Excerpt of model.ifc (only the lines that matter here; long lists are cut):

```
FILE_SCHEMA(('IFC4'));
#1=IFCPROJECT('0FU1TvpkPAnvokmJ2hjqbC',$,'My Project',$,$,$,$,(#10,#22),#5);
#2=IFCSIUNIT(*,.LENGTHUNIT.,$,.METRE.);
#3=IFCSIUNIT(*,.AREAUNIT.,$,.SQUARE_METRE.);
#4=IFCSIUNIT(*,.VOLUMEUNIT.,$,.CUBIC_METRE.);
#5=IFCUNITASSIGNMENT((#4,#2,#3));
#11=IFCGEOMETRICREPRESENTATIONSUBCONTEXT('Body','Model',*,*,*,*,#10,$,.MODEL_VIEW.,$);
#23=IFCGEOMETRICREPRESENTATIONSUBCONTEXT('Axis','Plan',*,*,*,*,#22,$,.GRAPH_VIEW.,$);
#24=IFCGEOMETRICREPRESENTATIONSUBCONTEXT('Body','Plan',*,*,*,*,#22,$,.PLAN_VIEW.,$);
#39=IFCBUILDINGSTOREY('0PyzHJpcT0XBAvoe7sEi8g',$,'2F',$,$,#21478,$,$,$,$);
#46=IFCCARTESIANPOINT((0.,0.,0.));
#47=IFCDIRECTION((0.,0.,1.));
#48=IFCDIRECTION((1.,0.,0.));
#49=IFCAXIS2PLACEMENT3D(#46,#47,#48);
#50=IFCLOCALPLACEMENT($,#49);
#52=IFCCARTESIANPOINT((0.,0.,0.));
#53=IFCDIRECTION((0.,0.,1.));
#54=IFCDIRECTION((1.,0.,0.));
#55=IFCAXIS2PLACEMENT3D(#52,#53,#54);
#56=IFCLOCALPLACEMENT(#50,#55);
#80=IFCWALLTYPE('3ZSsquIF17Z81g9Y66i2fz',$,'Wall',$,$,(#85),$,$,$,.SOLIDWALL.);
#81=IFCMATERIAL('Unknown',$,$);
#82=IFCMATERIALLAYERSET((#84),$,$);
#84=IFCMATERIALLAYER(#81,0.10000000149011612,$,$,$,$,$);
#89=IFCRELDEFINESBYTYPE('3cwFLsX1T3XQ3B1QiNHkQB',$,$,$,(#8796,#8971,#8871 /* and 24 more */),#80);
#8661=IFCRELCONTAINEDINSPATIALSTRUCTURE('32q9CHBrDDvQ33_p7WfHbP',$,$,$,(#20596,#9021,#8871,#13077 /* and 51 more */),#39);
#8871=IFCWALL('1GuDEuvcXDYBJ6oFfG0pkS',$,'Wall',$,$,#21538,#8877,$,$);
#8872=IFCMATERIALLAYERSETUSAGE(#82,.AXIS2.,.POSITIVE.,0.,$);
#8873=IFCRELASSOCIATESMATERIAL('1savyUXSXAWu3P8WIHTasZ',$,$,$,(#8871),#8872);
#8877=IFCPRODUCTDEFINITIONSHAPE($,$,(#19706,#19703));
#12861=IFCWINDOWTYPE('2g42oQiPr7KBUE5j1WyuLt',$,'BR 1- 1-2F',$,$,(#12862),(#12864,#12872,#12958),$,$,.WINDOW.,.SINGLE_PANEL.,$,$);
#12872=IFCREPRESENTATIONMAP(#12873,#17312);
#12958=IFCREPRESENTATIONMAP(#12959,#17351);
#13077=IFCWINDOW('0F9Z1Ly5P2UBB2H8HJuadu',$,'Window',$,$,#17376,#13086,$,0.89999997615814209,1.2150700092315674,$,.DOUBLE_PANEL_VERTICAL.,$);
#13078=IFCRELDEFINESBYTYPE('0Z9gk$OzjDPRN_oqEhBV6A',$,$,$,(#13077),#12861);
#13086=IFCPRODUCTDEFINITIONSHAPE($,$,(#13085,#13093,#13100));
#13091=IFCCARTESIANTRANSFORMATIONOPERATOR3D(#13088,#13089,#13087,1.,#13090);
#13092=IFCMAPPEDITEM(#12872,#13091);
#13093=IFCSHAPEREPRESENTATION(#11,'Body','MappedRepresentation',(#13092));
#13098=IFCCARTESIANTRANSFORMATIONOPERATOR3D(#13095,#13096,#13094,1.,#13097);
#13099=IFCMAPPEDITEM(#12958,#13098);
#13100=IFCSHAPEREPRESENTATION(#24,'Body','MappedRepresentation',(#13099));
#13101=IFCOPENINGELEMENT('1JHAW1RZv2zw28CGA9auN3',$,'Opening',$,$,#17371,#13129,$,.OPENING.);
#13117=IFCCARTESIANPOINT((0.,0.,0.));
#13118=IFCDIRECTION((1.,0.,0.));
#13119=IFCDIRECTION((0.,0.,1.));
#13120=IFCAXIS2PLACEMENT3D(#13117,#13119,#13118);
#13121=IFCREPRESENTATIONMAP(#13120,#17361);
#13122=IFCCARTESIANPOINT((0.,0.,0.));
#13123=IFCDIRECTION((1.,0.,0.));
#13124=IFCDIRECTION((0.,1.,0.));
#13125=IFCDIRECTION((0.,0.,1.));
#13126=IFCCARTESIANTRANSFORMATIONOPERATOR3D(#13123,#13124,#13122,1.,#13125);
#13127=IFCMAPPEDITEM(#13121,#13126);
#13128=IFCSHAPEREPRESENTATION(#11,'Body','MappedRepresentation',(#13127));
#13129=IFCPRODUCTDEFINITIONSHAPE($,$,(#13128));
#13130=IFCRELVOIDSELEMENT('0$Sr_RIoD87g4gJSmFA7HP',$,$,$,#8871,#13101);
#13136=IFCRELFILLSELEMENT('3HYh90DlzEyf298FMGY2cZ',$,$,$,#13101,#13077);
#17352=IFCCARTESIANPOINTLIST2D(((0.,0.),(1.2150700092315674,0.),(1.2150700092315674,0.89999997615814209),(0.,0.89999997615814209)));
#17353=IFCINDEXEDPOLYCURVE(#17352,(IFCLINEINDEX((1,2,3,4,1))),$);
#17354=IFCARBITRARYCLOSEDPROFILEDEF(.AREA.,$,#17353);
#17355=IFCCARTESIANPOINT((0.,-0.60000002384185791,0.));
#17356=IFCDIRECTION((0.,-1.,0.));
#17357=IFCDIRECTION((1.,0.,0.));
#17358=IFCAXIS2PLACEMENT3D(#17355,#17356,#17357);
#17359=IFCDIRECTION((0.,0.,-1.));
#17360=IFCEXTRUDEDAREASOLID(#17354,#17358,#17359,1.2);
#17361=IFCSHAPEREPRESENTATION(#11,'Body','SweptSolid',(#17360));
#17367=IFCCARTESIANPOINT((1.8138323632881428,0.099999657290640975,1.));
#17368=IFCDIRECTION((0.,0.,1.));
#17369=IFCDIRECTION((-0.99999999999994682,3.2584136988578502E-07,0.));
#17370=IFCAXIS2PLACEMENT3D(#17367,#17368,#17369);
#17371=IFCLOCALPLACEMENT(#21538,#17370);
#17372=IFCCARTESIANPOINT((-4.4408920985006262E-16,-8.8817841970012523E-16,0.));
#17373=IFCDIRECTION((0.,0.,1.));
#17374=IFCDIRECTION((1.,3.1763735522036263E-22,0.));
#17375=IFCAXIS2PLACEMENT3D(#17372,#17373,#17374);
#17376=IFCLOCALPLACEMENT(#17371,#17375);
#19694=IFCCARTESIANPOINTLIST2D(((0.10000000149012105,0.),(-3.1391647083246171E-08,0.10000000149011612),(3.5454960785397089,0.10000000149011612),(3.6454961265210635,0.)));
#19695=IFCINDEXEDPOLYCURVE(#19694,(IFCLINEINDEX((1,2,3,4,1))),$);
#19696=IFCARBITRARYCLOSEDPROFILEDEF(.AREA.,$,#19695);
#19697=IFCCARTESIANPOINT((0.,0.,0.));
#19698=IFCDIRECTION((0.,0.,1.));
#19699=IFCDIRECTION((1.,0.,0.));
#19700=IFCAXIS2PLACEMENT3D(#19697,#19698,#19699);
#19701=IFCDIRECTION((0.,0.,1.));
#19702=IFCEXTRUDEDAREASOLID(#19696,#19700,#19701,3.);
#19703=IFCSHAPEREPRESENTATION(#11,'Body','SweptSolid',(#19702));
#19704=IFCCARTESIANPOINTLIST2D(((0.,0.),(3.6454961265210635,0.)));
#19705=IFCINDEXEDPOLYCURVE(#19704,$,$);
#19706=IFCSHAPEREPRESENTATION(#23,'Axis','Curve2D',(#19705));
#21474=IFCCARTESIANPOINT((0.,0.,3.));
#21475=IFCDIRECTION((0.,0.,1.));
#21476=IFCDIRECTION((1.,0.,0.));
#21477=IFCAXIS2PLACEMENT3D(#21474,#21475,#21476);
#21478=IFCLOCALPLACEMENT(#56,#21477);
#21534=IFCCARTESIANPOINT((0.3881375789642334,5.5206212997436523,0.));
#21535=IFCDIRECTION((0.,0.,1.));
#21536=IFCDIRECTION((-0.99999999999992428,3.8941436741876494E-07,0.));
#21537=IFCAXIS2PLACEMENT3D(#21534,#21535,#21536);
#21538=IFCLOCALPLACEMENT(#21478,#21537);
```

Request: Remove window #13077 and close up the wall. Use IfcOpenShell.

```python
import ifcopenshell
import ifcopenshell.api.feature
import ifcopenshell.api.root
import ifcopenshell.geom
import ifcopenshell.util.shape

model = ifcopenshell.open("model.ifc")
settings = ifcopenshell.geom.settings()


def volume(element):
    """Net volume in cubic metres, openings subtracted."""
    shape = ifcopenshell.geom.create_shape(settings, element)
    return ifcopenshell.util.shape.get_volume(shape.geometry)


window = model.by_id(13077)
opening = window.FillsVoids[0].RelatingOpeningElement
wall = opening.VoidsElements[0].RelatingBuildingElement
before = volume(wall)

ifcopenshell.api.root.remove_product(model, product=window)
ifcopenshell.api.feature.remove_feature(model, feature=opening)

after = volume(wall)

print(f"wall volume {before:.3f} -> {after:.3f} m3")

model.write("model_v2.ifc")
```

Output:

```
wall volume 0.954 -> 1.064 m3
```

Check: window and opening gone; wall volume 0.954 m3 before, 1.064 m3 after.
